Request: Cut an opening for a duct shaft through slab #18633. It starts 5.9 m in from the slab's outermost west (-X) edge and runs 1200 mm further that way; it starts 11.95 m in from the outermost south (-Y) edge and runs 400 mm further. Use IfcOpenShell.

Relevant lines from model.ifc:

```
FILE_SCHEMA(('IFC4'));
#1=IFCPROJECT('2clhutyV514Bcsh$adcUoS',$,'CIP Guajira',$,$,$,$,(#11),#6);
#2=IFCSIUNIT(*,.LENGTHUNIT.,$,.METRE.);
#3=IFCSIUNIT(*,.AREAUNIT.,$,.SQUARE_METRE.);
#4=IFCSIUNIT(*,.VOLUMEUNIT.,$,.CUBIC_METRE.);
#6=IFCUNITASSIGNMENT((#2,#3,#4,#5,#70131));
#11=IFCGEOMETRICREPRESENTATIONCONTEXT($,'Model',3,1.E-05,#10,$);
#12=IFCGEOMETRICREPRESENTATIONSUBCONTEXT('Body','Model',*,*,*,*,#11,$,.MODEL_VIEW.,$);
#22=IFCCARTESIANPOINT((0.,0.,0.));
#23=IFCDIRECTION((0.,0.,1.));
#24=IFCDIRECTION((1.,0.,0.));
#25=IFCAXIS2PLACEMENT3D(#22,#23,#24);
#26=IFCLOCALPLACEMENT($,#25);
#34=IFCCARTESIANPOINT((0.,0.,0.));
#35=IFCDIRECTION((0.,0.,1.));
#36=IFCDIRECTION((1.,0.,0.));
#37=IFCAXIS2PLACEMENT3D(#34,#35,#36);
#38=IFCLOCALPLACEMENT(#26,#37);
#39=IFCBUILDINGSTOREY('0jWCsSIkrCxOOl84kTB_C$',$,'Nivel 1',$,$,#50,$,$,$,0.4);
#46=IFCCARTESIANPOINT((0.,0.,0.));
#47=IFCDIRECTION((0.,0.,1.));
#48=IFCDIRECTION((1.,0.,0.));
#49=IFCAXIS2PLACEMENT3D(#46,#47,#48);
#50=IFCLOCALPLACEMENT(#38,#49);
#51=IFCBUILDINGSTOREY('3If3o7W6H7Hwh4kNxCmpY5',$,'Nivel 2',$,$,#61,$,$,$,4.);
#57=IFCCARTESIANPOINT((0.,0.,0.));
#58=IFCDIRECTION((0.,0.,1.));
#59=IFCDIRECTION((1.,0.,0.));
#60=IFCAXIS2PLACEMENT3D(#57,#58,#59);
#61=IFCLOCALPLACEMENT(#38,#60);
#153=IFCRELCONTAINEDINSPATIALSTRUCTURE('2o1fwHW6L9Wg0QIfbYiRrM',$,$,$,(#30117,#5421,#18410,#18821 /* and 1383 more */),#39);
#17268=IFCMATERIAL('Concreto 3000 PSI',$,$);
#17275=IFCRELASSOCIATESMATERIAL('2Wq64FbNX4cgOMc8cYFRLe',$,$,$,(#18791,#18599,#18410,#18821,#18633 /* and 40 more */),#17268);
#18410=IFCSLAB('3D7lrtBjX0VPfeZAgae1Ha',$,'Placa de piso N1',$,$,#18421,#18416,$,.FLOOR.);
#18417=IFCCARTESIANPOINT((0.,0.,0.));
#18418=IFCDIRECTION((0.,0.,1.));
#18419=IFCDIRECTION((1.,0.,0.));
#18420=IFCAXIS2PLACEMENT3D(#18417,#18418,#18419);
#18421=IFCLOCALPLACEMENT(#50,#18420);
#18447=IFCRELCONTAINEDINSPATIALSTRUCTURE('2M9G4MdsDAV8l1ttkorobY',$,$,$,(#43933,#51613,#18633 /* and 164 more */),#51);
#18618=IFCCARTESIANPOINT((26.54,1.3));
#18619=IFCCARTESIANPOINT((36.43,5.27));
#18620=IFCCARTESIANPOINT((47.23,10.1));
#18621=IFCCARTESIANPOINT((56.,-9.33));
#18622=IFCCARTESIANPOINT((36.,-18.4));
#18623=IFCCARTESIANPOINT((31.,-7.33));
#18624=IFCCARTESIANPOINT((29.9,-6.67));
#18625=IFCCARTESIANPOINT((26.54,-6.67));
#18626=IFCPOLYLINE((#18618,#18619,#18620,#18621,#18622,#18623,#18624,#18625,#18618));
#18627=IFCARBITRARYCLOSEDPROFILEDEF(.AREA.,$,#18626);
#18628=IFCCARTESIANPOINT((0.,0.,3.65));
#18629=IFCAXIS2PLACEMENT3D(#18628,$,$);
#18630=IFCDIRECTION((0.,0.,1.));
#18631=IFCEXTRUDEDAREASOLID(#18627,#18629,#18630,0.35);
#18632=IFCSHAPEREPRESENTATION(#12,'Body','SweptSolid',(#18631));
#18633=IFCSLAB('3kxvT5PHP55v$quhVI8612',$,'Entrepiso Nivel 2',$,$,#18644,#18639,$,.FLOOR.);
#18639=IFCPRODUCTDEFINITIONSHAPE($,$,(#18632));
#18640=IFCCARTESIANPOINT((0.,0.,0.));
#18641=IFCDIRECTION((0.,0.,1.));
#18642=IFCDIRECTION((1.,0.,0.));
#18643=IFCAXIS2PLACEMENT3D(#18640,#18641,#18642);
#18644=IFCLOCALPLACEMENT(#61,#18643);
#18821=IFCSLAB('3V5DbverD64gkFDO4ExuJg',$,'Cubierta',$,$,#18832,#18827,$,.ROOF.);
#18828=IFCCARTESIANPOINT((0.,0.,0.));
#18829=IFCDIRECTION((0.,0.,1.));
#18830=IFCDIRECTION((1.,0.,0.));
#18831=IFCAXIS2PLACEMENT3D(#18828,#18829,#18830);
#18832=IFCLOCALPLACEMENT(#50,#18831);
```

```python
import numpy as np
import ifcopenshell
import ifcopenshell.api.feature
import ifcopenshell.api.geometry
import ifcopenshell.api.root
import ifcopenshell.geom
import ifcopenshell.util.placement
import ifcopenshell.util.representation
import ifcopenshell.util.shape
import ifcopenshell.util.unit

model = ifcopenshell.open("model.ifc")
unit_scale = ifcopenshell.util.unit.calculate_unit_scale(model)
settings = ifcopenshell.geom.settings()


def volume(element):
    """Net volume in cubic metres, openings subtracted."""
    shape = ifcopenshell.geom.create_shape(settings, element)
    return ifcopenshell.util.shape.get_volume(shape.geometry)


slab = model.by_guid("3kxvT5PHP55v$quhVI8612")
before = volume(slab)

# Extent in the slab's own axes, in metres. The edges named are its -X and -Y sides.
slab_shape = ifcopenshell.geom.create_shape(settings, slab)
vertices = ifcopenshell.util.shape.get_vertices(slab_shape.geometry)
x_min, y_min, bottom = vertices.min(axis=0)
top = vertices[:, 2].max()

opening = ifcopenshell.api.root.create_entity(model, ifc_class="IfcOpeningElement", name="Duct shaft opening", predefined_type="OPENING")
context = ifcopenshell.util.representation.get_context(model, "Model", "Body", "MODEL_VIEW")
width, depth = 1.2, 0.4
outline = [(0.0, 0.0), (width, 0.0), (width, depth), (0.0, depth), (0.0, 0.0)]
# Overshoot both faces by 50 mm so the cut is clean.
shape = ifcopenshell.api.geometry.add_slab_representation(
    model, context=context, depth=top - bottom + 0.1, polyline=outline
)
ifcopenshell.api.geometry.assign_representation(model, product=opening, representation=shape)

matrix = ifcopenshell.util.placement.get_local_placement(slab.ObjectPlacement)
matrix[:, 3] = matrix @ np.append(np.array([x_min + 5.9, y_min + 11.95, bottom - 0.05]) / unit_scale, 1.0)
ifcopenshell.api.geometry.edit_object_placement(model, product=opening, matrix=matrix, is_si=False)
ifcopenshell.api.feature.add_feature(model, feature=opening, element=slab)

after = volume(slab)

print(f"slab volume {before:.3f} -> {after:.3f} m3")

model.write("model_edited.ifc")
```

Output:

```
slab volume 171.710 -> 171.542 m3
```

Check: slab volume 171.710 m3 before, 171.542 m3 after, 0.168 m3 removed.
